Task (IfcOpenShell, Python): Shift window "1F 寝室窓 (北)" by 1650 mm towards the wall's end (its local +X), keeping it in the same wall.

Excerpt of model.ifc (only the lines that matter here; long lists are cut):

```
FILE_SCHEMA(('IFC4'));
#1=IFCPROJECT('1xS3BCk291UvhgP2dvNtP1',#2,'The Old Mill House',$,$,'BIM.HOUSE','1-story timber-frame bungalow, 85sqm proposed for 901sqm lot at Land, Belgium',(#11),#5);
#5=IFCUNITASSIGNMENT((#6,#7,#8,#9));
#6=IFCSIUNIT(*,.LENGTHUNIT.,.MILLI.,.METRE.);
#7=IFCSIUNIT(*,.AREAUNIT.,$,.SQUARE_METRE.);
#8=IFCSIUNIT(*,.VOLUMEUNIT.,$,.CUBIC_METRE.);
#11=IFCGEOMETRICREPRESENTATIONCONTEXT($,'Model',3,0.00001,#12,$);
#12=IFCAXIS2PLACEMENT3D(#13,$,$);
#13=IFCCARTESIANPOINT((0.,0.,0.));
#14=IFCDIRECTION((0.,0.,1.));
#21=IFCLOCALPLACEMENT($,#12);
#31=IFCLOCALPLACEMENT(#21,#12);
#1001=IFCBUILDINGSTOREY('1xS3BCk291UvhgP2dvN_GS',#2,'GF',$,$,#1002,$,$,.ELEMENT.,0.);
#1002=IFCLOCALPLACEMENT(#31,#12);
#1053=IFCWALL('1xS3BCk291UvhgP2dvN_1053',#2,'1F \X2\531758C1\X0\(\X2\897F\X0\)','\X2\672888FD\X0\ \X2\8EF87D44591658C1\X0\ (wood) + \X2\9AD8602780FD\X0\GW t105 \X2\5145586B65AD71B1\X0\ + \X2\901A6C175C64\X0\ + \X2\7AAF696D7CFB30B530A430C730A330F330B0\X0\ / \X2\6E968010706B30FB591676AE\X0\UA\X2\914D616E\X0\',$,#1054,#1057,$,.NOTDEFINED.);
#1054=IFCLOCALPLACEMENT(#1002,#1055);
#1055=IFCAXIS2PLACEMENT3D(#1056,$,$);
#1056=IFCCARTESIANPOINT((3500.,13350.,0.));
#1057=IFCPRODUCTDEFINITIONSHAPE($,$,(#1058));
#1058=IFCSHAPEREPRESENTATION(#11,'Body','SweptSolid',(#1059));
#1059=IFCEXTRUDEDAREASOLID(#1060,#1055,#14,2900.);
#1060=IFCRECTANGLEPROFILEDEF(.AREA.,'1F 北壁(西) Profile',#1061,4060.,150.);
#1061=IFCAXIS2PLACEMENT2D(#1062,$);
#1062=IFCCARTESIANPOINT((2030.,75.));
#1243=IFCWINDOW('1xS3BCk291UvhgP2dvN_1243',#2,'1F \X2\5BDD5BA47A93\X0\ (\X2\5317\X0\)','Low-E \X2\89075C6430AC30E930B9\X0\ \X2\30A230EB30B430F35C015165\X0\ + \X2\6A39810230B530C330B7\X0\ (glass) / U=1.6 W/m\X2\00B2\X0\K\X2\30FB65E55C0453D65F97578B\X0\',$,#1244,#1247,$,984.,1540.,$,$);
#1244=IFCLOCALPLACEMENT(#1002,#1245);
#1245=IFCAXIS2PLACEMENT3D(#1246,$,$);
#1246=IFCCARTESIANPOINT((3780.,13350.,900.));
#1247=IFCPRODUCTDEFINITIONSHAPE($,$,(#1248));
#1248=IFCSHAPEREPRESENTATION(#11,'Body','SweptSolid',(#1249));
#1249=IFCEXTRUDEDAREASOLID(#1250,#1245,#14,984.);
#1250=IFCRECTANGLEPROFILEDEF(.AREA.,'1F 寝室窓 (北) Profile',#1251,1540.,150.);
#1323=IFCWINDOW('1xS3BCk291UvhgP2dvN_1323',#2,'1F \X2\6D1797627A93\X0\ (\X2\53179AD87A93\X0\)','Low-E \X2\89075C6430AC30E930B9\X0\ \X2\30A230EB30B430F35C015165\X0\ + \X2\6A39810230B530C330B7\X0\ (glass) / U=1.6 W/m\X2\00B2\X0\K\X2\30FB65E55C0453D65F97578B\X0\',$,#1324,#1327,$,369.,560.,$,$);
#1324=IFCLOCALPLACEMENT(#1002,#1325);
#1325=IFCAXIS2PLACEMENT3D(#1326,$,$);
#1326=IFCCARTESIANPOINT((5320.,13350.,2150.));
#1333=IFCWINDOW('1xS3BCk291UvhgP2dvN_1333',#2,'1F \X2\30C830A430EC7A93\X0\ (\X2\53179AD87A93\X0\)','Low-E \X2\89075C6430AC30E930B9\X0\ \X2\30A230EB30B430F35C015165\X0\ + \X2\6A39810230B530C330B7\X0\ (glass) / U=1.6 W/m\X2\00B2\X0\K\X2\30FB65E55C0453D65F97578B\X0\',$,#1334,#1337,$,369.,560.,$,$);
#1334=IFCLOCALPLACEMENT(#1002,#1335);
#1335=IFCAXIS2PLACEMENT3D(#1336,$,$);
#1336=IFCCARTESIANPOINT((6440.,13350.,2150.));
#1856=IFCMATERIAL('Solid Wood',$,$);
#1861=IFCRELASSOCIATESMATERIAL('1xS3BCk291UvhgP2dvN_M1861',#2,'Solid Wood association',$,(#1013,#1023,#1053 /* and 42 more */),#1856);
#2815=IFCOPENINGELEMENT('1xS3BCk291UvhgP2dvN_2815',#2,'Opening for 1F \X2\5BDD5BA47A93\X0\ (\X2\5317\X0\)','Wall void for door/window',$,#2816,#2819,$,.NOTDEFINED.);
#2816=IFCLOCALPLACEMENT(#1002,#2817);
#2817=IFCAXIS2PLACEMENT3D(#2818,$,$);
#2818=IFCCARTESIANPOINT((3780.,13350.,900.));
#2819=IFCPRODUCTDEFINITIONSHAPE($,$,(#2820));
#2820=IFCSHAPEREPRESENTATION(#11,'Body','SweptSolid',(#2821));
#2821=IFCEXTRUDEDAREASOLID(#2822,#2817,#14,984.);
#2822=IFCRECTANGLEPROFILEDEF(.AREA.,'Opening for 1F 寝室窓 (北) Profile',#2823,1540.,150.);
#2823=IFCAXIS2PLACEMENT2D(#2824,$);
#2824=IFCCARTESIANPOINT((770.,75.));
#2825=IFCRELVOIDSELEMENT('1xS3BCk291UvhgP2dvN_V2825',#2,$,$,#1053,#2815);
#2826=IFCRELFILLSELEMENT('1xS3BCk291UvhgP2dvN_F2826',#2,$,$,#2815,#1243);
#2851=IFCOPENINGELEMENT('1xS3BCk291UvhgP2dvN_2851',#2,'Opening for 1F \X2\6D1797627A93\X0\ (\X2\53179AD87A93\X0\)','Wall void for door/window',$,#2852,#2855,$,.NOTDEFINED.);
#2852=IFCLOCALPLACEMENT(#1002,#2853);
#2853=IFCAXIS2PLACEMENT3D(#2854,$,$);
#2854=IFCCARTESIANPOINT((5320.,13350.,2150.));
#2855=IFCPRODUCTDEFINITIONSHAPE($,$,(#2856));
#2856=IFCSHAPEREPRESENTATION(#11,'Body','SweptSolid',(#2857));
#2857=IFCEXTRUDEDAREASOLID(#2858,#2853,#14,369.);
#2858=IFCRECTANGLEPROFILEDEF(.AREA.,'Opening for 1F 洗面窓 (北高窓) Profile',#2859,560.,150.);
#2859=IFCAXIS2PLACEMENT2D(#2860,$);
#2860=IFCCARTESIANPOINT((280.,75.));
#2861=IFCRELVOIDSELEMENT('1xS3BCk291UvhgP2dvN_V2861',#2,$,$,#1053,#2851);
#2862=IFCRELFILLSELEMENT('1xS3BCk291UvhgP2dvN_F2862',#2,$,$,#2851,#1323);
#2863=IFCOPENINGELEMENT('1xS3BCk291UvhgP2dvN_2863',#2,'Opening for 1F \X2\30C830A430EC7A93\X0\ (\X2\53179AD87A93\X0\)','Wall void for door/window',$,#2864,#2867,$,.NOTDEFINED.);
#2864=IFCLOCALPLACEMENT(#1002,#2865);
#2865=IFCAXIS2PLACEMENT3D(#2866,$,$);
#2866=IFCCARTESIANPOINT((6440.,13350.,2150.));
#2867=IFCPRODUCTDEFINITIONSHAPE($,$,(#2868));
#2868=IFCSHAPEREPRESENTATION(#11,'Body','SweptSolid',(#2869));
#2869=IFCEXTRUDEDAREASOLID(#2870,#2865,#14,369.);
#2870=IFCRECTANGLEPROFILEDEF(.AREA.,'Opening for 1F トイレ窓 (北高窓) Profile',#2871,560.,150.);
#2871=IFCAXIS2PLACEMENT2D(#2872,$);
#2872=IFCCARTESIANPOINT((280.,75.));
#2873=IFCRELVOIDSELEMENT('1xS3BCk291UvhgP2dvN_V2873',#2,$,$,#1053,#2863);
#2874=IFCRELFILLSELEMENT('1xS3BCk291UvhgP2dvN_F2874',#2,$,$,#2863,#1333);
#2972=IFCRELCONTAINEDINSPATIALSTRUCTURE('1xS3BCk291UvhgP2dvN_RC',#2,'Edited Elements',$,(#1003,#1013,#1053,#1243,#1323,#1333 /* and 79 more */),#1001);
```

```python
import ifcopenshell
import ifcopenshell.api.geometry
import ifcopenshell.util.placement
import ifcopenshell.util.unit

model = ifcopenshell.open("model.ifc")
unit_scale = ifcopenshell.util.unit.calculate_unit_scale(model)

window = model.by_guid("1xS3BCk291UvhgP2dvN_1243")
opening = window.FillsVoids[0].RelatingOpeningElement
wall = opening.VoidsElements[0].RelatingBuildingElement

wall_matrix = ifcopenshell.util.placement.get_local_placement(wall.ObjectPlacement)
shift = wall_matrix[:3, 0] * 1.65 / unit_scale
before = ifcopenshell.util.placement.get_local_placement(window.ObjectPlacement)[:3, 3].copy()

# The window is not placed relative to its opening, so move both.
for product in (opening, window):
    matrix = ifcopenshell.util.placement.get_local_placement(product.ObjectPlacement)
    matrix[:3, 3] += shift
    ifcopenshell.api.geometry.edit_object_placement(model, product=product, matrix=matrix, is_si=False)

after = ifcopenshell.util.placement.get_local_placement(window.ObjectPlacement)[:3, 3]
print("window moved by", (after - before).round(3) + 0.0)

model.write("model_edited.ifc")
```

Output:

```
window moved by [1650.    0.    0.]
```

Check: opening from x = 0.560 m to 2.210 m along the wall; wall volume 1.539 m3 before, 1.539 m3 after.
